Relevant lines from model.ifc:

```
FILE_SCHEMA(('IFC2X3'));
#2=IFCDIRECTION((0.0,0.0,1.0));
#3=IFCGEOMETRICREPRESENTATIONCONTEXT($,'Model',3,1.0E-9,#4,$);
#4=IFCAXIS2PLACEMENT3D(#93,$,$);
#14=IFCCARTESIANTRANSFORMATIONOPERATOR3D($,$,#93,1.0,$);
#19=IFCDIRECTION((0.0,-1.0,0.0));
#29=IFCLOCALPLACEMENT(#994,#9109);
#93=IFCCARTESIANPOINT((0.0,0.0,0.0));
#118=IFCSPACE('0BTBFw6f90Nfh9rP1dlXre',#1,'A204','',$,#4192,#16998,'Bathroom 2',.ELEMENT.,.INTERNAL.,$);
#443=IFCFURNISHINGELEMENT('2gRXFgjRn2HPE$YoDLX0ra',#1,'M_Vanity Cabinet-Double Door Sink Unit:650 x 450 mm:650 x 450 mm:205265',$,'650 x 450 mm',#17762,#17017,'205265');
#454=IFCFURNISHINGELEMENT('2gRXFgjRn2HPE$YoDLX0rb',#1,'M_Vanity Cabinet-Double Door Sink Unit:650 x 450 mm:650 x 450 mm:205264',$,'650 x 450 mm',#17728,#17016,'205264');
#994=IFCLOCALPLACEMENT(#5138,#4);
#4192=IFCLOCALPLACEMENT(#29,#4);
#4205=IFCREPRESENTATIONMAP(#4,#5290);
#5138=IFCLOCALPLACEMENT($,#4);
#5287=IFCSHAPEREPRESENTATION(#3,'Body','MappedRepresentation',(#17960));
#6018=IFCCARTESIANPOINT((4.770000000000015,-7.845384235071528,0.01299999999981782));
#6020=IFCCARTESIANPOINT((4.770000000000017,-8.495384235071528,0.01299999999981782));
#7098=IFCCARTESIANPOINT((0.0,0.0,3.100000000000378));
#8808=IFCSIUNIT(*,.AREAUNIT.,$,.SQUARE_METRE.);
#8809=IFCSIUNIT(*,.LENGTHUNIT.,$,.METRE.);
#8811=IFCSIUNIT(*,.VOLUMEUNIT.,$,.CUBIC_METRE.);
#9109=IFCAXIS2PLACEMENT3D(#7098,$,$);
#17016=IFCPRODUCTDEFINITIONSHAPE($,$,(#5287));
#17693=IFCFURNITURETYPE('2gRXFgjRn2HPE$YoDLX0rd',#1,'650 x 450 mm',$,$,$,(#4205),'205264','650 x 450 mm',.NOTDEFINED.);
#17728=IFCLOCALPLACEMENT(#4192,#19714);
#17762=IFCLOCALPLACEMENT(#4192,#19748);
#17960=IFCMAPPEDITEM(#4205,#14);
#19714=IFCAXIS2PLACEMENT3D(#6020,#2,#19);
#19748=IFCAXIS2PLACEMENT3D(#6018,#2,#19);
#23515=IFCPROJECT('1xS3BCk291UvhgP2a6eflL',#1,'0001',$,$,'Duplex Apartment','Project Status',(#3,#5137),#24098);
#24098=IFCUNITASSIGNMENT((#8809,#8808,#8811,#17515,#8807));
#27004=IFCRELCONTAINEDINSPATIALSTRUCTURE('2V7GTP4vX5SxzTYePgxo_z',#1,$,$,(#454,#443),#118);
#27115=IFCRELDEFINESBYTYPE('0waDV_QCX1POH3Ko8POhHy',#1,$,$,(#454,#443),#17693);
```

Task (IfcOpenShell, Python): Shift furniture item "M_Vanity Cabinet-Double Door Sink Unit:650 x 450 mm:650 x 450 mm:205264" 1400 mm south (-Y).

```python
import ifcopenshell
import ifcopenshell.api.geometry
import ifcopenshell.util.placement
import ifcopenshell.util.unit

model = ifcopenshell.open("model.ifc")
unit_scale = ifcopenshell.util.unit.calculate_unit_scale(model)

item = model.by_id(454)
matrix = ifcopenshell.util.placement.get_local_placement(item.ObjectPlacement)
matrix[1, 3] -= 1.4 / unit_scale
ifcopenshell.api.geometry.edit_object_placement(model, product=item, matrix=matrix, is_si=False)

print(ifcopenshell.util.placement.get_local_placement(item.ObjectPlacement).round(3) + 0.0)

model.write("model_v2.ifc")
```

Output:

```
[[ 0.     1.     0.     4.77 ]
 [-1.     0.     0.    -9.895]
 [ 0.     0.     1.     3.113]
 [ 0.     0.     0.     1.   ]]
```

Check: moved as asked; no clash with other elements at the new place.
